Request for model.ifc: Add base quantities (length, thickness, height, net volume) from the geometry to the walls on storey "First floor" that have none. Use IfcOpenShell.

First a look at what the model holds.

```python
import ifcopenshell
import ifcopenshell.util.element
import ifcopenshell.util.unit

model = ifcopenshell.open("model.ifc")
print(model.schema)
for unit_type in ("LENGTHUNIT", "AREAUNIT", "VOLUMEUNIT"):
    print(unit_type, ifcopenshell.util.unit.calculate_unit_scale(model, unit_type))
storey = next(s for s in model.by_type("IfcBuildingStorey") if s.Name == "First floor")
walls = [e for e in ifcopenshell.util.element.get_decomposition(storey) if e.is_a("IfcWall")]
for e in sorted(walls, key=lambda e: e.id()):
    print(e.id(), e.is_a(), e.Name, list(ifcopenshell.util.element.get_psets(e, qtos_only=True)), sep=" | ")
```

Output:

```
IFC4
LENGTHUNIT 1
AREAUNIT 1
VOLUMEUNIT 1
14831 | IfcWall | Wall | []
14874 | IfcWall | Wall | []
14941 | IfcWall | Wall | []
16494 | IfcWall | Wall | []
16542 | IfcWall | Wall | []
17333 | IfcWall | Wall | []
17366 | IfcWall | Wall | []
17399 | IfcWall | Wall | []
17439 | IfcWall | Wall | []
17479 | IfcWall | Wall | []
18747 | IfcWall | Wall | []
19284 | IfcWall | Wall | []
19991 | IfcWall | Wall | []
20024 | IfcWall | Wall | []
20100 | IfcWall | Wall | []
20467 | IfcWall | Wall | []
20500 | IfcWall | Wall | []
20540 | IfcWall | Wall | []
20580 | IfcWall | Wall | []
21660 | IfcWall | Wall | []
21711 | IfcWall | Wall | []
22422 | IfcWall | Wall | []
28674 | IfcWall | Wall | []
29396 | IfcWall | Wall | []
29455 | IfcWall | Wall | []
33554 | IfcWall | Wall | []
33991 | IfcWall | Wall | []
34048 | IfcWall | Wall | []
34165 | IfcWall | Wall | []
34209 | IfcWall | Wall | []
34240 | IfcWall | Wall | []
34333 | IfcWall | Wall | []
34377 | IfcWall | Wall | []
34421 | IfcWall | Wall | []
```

```python
import ifcopenshell
import ifcopenshell.api.pset
import ifcopenshell.geom
import ifcopenshell.util.element
import ifcopenshell.util.shape
import ifcopenshell.util.unit

model = ifcopenshell.open("model.ifc")
unit_scale = ifcopenshell.util.unit.calculate_unit_scale(model)
volume_scale = ifcopenshell.util.unit.calculate_unit_scale(model, "VOLUMEUNIT")
settings = ifcopenshell.geom.settings()

storey = next(s for s in model.by_type("IfcBuildingStorey") if s.Name == "First floor")
walls = [e for e in ifcopenshell.util.element.get_decomposition(storey) if e.is_a("IfcWall")]

for e in sorted(walls, key=lambda e: e.id()):
    if ifcopenshell.util.element.get_psets(e, qtos_only=True, should_inherit=False):
        continue
    # Geometry comes back in metres, in the element's own axes.
    shape = ifcopenshell.geom.create_shape(settings, e)
    values = {
        "Length": ifcopenshell.util.shape.get_x(shape.geometry) / unit_scale,
        "Width": ifcopenshell.util.shape.get_y(shape.geometry) / unit_scale,
        "Height": ifcopenshell.util.shape.get_z(shape.geometry) / unit_scale,
        "NetVolume": ifcopenshell.util.shape.get_volume(shape.geometry) / volume_scale,
    }
    qto = ifcopenshell.api.pset.add_qto(model, product=e, name="Qto_WallBaseQuantities")
    ifcopenshell.api.pset.edit_qto(model, qto=qto, properties=values)
    print(e.id(), {k: round(v, 3) for k, v in values.items()})

model.write("model_edited.ifc")
```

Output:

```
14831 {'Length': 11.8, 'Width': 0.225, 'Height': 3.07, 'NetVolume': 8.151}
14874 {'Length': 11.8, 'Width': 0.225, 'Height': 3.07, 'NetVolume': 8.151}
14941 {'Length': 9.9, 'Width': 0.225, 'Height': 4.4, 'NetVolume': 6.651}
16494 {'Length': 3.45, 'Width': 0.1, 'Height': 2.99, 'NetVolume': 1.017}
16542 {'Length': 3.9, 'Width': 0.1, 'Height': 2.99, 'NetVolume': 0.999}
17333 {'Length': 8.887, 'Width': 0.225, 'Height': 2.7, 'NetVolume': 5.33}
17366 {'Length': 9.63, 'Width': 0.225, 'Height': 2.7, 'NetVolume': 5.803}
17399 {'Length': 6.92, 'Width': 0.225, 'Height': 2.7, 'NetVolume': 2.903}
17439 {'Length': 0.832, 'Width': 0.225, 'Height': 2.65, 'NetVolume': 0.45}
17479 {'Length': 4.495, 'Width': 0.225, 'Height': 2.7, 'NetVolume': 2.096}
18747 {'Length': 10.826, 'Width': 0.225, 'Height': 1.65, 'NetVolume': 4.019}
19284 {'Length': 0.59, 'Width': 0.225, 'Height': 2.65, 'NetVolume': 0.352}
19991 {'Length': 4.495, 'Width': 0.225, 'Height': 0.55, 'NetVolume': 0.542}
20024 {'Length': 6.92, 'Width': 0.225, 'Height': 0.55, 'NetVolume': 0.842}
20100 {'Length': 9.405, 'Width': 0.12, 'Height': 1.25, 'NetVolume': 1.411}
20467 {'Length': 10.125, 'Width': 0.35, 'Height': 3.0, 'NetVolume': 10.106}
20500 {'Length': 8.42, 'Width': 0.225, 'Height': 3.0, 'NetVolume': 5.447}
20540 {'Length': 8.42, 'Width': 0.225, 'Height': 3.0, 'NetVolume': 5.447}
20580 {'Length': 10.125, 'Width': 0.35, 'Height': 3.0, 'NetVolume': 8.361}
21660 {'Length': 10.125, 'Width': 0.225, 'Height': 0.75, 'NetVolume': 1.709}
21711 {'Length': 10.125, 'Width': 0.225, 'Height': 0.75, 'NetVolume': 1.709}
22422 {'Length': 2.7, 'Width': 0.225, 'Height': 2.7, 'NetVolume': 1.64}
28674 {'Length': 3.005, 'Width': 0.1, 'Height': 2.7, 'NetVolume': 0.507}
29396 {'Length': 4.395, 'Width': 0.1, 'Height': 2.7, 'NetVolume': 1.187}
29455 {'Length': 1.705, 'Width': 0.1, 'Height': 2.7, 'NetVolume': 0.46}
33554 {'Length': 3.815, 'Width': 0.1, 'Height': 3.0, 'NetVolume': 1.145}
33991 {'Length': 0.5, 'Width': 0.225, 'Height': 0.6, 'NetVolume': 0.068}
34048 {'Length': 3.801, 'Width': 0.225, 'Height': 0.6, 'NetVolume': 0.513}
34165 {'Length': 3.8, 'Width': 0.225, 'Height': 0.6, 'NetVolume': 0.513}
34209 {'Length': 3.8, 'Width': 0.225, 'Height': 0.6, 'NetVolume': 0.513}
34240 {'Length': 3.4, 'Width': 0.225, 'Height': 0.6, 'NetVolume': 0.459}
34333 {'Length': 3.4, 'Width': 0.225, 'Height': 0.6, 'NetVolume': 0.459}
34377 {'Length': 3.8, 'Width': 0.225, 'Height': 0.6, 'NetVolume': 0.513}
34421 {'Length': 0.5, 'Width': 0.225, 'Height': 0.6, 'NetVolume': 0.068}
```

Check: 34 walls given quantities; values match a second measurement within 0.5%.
